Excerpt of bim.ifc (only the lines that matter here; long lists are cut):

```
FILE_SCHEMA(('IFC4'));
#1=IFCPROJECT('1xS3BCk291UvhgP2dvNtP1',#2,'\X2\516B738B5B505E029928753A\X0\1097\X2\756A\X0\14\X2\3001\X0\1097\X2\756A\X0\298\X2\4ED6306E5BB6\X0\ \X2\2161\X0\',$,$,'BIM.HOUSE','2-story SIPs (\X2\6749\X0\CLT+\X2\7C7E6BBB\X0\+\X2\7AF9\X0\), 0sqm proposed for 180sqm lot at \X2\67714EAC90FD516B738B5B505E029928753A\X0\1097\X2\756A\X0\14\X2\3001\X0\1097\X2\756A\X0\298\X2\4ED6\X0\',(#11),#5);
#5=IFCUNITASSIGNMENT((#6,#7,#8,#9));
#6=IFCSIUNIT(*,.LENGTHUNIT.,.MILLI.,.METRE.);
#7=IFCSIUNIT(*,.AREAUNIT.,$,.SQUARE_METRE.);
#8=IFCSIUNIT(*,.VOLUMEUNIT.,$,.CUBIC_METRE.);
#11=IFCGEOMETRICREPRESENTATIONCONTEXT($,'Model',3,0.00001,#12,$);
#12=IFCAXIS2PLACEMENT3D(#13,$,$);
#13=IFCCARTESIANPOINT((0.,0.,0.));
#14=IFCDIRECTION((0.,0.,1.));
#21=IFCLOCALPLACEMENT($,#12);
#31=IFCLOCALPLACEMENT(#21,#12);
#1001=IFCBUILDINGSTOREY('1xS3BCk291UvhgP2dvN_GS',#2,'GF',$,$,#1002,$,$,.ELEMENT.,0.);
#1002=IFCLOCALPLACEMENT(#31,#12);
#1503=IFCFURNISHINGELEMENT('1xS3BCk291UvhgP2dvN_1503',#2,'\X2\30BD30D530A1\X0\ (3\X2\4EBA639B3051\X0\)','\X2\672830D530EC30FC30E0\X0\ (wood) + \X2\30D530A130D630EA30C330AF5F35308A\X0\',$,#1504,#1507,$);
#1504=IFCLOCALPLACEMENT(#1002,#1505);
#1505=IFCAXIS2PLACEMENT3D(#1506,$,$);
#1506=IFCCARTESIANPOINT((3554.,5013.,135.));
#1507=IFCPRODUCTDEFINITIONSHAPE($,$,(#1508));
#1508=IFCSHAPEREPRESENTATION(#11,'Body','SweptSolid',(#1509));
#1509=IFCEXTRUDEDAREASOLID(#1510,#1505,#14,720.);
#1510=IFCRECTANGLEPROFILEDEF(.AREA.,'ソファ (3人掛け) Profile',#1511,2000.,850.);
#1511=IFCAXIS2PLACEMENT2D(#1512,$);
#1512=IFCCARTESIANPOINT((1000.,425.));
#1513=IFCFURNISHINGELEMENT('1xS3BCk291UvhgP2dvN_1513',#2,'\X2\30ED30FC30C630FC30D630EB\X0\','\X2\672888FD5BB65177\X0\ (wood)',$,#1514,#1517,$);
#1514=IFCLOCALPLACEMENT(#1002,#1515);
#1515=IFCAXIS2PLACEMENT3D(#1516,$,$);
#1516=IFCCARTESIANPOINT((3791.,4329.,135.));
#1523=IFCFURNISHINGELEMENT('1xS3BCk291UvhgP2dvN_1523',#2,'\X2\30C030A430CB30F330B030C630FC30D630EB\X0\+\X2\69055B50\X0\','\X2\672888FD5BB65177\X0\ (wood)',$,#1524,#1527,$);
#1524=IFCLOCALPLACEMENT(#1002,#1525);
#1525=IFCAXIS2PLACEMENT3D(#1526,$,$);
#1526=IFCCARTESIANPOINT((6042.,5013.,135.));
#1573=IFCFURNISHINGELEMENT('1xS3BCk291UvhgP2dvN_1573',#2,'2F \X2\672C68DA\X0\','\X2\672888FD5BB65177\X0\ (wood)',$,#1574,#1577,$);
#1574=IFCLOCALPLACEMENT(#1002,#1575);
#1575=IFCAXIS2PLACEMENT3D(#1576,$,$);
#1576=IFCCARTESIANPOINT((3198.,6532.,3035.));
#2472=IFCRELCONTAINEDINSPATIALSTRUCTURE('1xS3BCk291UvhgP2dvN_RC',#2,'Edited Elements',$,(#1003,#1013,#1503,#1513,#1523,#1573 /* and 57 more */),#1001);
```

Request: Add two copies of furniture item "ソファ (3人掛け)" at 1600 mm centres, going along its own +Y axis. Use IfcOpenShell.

```python
import ifcopenshell
import ifcopenshell.api.geometry
import ifcopenshell.api.root
import ifcopenshell.util.element
import ifcopenshell.util.placement
import ifcopenshell.util.unit

model = ifcopenshell.open("bim.ifc")
unit_scale = ifcopenshell.util.unit.calculate_unit_scale(model)


def reuse_history(source, copy):
    """copy_class also copies each property set's owner history, people and application; keep the originals."""
    for rel in copy.IsDefinedBy:
        if rel.is_a("IfcRelDefinesByProperties") and (history := rel.RelatingPropertyDefinition.OwnerHistory):
            rel.RelatingPropertyDefinition.OwnerHistory = source.OwnerHistory
            ifcopenshell.util.element.remove_deep2(model, history)


source = model.by_id(1503)
base = ifcopenshell.util.placement.get_local_placement(source.ObjectPlacement)
step = base[:3, 1] * 1.6 / unit_scale

for i in range(1, 3):
    copy = ifcopenshell.api.root.copy_class(model, product=source)
    copy.Representation = ifcopenshell.util.element.copy_deep(
        model, source.Representation, exclude=["IfcGeometricRepresentationContext", "IfcRepresentationMap"]
    )
    reuse_history(source, copy)
    matrix = base.copy()
    matrix[:3, 3] += i * step
    print("added at", matrix[:3, 3].round(3) + 0.0)
    ifcopenshell.api.geometry.edit_object_placement(model, product=copy, matrix=matrix, is_si=False)

model.write("bim_v2.ifc")
```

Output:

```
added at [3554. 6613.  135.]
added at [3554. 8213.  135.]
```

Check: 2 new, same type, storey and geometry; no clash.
